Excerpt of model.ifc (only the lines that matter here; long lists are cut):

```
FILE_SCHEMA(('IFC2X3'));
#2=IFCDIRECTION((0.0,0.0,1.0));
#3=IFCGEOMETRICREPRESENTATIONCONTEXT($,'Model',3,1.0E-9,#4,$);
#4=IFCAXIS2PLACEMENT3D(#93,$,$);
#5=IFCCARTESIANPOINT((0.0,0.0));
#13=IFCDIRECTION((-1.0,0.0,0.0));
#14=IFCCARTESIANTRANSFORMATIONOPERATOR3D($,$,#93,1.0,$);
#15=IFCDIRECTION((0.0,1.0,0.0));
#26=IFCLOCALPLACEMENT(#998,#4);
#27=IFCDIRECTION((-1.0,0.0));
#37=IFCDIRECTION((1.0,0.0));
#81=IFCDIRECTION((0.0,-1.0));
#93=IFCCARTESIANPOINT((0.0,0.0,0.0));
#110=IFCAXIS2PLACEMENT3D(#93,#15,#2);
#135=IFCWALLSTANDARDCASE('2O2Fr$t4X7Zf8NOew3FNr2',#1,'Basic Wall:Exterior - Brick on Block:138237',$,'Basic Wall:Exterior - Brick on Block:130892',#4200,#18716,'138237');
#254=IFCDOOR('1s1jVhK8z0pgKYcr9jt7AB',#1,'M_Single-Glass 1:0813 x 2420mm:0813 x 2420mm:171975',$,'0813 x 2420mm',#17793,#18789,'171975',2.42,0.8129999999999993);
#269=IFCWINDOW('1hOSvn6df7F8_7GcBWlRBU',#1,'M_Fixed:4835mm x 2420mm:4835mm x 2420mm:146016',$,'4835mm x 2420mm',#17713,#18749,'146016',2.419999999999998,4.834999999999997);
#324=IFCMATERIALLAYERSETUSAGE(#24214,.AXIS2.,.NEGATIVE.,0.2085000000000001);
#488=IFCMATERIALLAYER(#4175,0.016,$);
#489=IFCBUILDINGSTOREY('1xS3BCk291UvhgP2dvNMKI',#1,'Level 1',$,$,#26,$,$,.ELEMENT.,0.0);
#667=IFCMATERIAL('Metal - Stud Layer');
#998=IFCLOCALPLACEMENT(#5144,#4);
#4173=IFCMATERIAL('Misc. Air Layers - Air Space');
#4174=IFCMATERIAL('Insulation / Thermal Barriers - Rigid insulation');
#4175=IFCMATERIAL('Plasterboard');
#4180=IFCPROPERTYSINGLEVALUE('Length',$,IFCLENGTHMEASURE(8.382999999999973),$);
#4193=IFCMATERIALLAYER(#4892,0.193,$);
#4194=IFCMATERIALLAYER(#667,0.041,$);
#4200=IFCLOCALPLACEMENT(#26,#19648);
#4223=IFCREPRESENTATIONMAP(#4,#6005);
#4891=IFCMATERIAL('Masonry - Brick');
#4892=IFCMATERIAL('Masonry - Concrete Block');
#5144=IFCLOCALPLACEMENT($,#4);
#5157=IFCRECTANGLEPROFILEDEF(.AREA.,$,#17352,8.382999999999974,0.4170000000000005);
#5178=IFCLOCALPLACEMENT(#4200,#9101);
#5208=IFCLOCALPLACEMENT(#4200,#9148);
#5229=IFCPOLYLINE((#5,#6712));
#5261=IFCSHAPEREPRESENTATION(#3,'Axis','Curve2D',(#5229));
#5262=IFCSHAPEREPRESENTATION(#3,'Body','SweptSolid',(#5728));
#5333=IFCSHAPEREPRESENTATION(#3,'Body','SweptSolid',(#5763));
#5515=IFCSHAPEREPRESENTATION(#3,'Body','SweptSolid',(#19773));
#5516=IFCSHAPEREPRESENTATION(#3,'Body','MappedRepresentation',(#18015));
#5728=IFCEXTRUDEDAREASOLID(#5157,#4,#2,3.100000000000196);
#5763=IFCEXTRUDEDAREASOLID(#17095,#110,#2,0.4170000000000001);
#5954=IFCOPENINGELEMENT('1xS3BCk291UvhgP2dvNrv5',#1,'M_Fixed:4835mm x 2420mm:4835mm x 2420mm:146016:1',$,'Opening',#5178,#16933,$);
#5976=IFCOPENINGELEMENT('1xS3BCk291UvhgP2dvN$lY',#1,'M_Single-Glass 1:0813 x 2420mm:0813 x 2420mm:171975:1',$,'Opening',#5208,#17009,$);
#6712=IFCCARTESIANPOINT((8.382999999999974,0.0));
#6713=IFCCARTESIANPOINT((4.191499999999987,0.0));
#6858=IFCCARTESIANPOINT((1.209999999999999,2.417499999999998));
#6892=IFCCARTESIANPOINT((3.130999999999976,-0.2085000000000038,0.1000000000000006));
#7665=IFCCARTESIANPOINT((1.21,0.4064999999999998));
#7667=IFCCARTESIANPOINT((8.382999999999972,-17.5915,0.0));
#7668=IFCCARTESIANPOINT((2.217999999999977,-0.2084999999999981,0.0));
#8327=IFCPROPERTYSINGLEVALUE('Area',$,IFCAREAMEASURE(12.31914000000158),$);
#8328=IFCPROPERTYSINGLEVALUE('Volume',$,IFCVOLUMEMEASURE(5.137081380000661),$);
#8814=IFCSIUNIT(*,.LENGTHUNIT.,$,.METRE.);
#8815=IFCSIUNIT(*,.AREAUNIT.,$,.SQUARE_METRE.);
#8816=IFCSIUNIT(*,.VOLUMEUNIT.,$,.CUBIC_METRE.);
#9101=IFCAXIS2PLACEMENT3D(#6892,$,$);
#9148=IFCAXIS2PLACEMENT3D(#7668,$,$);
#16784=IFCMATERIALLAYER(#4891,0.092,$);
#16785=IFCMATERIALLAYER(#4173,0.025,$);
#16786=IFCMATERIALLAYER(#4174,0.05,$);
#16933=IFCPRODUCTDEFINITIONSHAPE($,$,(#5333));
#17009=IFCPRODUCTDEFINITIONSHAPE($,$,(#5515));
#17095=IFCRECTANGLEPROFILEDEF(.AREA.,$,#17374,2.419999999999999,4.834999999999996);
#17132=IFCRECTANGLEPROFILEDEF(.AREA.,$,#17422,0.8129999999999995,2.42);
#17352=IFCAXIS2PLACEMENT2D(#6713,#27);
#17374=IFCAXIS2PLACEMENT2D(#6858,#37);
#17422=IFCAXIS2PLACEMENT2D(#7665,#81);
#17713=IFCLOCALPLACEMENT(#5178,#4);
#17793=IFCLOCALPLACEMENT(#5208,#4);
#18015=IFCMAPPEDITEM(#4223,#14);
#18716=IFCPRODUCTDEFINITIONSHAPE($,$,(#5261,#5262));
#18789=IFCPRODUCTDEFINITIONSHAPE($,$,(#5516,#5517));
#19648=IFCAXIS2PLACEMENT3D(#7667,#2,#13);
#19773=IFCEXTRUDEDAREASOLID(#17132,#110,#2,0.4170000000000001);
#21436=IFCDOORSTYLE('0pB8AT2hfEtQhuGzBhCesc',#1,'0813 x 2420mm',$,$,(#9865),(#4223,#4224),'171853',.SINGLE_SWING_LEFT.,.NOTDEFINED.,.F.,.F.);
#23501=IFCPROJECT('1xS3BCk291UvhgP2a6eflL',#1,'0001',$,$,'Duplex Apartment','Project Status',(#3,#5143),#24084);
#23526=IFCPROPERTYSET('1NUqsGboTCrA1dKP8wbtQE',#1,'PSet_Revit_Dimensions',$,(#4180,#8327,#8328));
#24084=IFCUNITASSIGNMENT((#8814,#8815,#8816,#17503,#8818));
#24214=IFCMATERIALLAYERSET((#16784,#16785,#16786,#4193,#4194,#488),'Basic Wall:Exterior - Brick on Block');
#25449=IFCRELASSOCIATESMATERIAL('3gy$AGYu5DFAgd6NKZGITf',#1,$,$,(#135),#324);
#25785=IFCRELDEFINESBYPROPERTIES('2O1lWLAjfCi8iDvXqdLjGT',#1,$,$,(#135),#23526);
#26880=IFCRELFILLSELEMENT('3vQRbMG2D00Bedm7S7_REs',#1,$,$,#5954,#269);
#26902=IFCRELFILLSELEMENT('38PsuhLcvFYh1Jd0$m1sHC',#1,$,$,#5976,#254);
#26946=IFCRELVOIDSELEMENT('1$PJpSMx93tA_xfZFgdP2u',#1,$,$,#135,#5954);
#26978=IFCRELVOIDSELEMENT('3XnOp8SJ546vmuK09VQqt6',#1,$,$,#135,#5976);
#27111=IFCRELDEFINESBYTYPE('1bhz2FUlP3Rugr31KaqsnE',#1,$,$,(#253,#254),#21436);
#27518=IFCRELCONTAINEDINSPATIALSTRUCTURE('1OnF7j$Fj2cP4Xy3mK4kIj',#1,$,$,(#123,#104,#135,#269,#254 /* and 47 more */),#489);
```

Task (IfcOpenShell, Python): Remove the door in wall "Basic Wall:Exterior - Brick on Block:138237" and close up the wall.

```python
import ifcopenshell
import ifcopenshell.api.feature
import ifcopenshell.api.pset
import ifcopenshell.api.root
import ifcopenshell.geom
import ifcopenshell.util.element
import ifcopenshell.util.shape
import ifcopenshell.util.unit

model = ifcopenshell.open("model.ifc")
area_scale = ifcopenshell.util.unit.calculate_unit_scale(model, "AREAUNIT")
volume_scale = ifcopenshell.util.unit.calculate_unit_scale(model, "VOLUMEUNIT")
settings = ifcopenshell.geom.settings()


def volume(element):
    """Net volume in cubic metres, openings subtracted."""
    shape = ifcopenshell.geom.create_shape(settings, element)
    return ifcopenshell.util.shape.get_volume(shape.geometry)


door = model.by_id(254)
opening = door.FillsVoids[0].RelatingOpeningElement
wall = opening.VoidsElements[0].RelatingBuildingElement
before = volume(wall)

ifcopenshell.api.root.remove_product(model, product=door)
ifcopenshell.api.feature.remove_feature(model, feature=opening)

after = volume(wall)
thickness = 0.417  # wall thickness in metres

# Update the wall's stored quantities.
pset = model.by_id(ifcopenshell.util.element.get_pset(wall, "PSet_Revit_Dimensions", should_inherit=False)["id"])
ifcopenshell.api.pset.edit_pset(model, pset=pset, properties={
    "Area": model.create_entity("IfcAreaMeasure", after / thickness / area_scale),
    "Volume": model.create_entity("IfcVolumeMeasure", after / volume_scale),
})

print(f"wall volume {before:.3f} -> {after:.3f} m3")

model.write("model_rev.ifc")
```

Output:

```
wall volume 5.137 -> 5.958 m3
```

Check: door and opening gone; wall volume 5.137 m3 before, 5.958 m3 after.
